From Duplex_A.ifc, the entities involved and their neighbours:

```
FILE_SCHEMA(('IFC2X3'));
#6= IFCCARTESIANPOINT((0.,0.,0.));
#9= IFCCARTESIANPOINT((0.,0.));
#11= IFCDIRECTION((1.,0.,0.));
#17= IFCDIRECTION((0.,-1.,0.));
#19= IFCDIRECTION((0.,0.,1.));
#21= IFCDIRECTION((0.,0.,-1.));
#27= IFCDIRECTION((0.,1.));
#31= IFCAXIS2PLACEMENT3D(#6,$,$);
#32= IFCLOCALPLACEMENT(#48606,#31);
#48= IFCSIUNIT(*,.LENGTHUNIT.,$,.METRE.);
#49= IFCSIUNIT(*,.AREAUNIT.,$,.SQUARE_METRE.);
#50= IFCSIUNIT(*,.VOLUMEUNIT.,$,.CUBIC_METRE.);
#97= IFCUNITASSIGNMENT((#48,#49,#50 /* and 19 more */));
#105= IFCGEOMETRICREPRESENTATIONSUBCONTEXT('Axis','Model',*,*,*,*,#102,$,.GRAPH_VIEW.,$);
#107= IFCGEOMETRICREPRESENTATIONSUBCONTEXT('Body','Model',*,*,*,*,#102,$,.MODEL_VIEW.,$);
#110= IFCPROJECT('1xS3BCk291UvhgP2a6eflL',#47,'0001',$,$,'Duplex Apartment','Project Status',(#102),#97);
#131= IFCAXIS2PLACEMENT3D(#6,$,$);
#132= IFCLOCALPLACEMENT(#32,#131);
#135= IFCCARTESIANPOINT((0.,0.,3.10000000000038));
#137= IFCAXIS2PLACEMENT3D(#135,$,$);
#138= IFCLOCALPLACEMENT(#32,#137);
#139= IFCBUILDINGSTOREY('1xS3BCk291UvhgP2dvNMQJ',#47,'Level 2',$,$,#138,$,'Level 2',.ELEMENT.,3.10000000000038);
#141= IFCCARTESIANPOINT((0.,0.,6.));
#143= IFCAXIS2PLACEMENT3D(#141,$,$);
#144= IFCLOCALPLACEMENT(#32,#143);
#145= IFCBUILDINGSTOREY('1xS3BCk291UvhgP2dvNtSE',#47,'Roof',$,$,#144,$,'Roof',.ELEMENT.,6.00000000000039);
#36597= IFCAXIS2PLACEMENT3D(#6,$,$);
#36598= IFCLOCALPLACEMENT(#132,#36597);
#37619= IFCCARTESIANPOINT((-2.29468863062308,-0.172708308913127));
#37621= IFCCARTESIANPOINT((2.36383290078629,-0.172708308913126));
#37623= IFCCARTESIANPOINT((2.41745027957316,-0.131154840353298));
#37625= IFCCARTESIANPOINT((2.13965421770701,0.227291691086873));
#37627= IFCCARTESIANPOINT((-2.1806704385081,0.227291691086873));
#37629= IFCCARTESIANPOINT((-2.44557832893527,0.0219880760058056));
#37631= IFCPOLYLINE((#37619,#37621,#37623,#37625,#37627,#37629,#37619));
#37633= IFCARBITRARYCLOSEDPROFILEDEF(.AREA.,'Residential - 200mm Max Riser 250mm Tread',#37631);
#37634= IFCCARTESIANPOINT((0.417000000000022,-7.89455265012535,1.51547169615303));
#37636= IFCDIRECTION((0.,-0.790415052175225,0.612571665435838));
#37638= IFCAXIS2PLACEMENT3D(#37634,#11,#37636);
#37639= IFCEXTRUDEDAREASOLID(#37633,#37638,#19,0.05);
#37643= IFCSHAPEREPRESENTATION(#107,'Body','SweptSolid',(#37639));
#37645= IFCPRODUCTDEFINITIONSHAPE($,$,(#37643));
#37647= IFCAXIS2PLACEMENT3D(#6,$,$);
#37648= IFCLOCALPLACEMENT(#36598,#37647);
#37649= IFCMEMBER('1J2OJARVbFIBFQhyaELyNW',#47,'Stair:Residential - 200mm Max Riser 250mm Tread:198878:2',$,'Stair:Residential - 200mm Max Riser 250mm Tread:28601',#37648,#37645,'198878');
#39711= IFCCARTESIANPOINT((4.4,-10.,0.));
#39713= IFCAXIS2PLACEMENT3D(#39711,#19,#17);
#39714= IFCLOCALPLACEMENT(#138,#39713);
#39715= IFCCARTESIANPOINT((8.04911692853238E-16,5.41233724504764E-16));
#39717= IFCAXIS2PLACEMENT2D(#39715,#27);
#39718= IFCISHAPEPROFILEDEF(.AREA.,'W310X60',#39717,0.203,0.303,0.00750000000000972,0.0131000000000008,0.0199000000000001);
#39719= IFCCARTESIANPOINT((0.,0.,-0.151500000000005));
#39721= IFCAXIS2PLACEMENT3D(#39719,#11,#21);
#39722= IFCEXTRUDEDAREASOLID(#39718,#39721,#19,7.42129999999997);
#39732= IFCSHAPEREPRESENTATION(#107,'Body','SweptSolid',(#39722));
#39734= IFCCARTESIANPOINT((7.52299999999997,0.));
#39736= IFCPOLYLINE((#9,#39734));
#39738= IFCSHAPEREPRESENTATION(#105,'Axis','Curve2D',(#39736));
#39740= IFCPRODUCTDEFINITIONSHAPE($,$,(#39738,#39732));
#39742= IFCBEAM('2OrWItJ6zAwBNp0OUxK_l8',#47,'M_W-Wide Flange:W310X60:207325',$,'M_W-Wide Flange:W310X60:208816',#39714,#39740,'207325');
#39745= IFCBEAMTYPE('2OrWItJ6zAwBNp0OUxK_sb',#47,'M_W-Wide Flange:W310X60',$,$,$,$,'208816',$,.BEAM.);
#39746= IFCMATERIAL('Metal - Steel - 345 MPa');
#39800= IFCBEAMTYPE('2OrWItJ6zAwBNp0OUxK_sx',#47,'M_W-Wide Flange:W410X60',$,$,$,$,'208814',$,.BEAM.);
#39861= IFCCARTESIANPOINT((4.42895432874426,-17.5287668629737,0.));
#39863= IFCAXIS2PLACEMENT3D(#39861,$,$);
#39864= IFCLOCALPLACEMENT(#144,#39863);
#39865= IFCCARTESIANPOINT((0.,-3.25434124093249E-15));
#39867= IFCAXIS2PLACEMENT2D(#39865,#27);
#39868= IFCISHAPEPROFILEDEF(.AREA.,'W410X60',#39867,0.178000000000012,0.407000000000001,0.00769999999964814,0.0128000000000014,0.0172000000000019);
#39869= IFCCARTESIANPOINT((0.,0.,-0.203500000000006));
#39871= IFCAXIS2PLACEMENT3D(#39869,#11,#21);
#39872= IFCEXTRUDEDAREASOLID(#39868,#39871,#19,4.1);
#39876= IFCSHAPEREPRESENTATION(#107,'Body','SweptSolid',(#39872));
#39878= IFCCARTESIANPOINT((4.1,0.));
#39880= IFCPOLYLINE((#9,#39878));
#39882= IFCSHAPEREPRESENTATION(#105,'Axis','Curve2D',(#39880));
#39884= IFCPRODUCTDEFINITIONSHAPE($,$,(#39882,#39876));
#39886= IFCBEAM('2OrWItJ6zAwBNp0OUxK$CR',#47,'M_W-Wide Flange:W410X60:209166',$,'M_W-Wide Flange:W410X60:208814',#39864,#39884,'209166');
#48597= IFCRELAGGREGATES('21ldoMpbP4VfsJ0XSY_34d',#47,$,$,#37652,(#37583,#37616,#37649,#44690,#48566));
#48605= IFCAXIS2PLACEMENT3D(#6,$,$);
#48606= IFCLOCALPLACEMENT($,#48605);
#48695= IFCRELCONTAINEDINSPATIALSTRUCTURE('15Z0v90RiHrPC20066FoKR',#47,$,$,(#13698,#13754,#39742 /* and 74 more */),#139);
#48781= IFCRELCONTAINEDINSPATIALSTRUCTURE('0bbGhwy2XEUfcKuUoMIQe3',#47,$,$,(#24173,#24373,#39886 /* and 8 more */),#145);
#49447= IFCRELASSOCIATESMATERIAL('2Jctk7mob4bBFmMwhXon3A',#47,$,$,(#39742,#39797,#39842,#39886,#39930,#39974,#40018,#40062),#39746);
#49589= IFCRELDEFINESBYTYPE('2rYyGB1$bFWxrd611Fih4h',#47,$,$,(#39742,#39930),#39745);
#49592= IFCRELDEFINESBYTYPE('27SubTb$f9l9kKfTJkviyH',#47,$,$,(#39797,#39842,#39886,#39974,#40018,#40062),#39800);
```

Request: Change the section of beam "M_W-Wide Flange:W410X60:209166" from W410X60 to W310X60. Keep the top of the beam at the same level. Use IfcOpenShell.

```python
import ifcopenshell
import ifcopenshell.api.type
import ifcopenshell.util.element
import ifcopenshell.util.representation

model = ifcopenshell.open("Duplex_A.ifc")

member = model.by_guid("2OrWItJ6zAwBNp0OUxK$CR")
source = next(p for p in model.by_type("IfcIShapeProfileDef") if p.ProfileName == "W310X60")

body = ifcopenshell.util.representation.get_representation(member, "Model", "Body")
solid = body.Items[0]
old_profile = solid.SweptArea

# Copy the section's sizes but keep this member's own profile position.
profile = ifcopenshell.util.element.copy(model, source)
# Profiles are centred, so shift by half the change in depth to hold the top.
shift = (old_profile.OverallDepth - profile.OverallDepth) / 2
x, y = old_profile.Position.Location.Coordinates
up = (-1.0, 0.0)  # upwards, in the solid's own plane
location = model.createIfcCartesianPoint((x + up[0] * shift, y + up[1] * shift))
profile.Position = model.createIfcAxis2Placement2D(location, old_profile.Position.RefDirection)
solid.SweptArea = profile
if not model.get_total_inverses(old_profile):
    ifcopenshell.util.element.remove_deep2(model, old_profile)

new_type = model.by_guid("2OrWItJ6zAwBNp0OUxK_sb")
ifcopenshell.api.type.assign_type(
    model, related_objects=[member], relating_type=new_type, should_map_representations=False
)
member.Name = member.Name.replace("W410X60", "W310X60")
member.ObjectType = "M_W-Wide Flange:W310X60:208814"

print(solid.SweptArea)

model.write("Duplex_A-out.ifc")
```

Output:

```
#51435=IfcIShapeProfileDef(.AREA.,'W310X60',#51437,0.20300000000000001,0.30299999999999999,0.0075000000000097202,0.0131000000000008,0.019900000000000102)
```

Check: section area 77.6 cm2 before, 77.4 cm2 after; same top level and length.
